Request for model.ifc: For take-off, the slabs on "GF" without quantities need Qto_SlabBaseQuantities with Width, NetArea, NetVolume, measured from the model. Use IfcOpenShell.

First a look at what the model holds.

```python
import ifcopenshell
import ifcopenshell.util.element
import ifcopenshell.util.unit

model = ifcopenshell.open("model.ifc")
print(model.schema)
for unit_type in ("LENGTHUNIT", "AREAUNIT", "VOLUMEUNIT"):
    print(unit_type, ifcopenshell.util.unit.calculate_unit_scale(model, unit_type))
storey = next(s for s in model.by_type("IfcBuildingStorey") if s.Name == "GF")
slabs = [e for e in ifcopenshell.util.element.get_decomposition(storey) if e.is_a("IfcSlab")]
for e in sorted(slabs, key=lambda e: e.id()):
    print(e.id(), e.is_a(), e.Name, list(ifcopenshell.util.element.get_psets(e, qtos_only=True)), sep=" | ")
```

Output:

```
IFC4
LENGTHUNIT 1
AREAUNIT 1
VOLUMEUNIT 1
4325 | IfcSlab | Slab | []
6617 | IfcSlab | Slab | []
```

```python
import ifcopenshell
import ifcopenshell.api.pset
import ifcopenshell.geom
import ifcopenshell.util.element
import ifcopenshell.util.shape
import ifcopenshell.util.unit

model = ifcopenshell.open("model.ifc")
unit_scale = ifcopenshell.util.unit.calculate_unit_scale(model)
area_scale = ifcopenshell.util.unit.calculate_unit_scale(model, "AREAUNIT")
volume_scale = ifcopenshell.util.unit.calculate_unit_scale(model, "VOLUMEUNIT")
settings = ifcopenshell.geom.settings()

storey = next(s for s in model.by_type("IfcBuildingStorey") if s.Name == "GF")
slabs = [e for e in ifcopenshell.util.element.get_decomposition(storey) if e.is_a("IfcSlab")]

for e in sorted(slabs, key=lambda e: e.id()):
    if ifcopenshell.util.element.get_psets(e, qtos_only=True, should_inherit=False):
        continue
    # Geometry comes back in metres, in the element's own axes.
    shape = ifcopenshell.geom.create_shape(settings, e)
    values = {
        "Width": ifcopenshell.util.shape.get_z(shape.geometry) / unit_scale,
        "NetArea": ifcopenshell.util.shape.get_footprint_area(shape.geometry) / area_scale,
        "NetVolume": ifcopenshell.util.shape.get_volume(shape.geometry) / volume_scale,
    }
    qto = ifcopenshell.api.pset.add_qto(model, product=e, name="Qto_SlabBaseQuantities")
    ifcopenshell.api.pset.edit_qto(model, qto=qto, properties=values)
    print(e.id(), {k: round(v, 3) for k, v in values.items()})

model.write("model_edited.ifc")
```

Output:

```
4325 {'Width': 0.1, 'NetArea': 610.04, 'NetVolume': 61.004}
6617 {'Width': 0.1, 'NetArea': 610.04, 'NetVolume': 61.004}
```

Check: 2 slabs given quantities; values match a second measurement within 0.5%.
